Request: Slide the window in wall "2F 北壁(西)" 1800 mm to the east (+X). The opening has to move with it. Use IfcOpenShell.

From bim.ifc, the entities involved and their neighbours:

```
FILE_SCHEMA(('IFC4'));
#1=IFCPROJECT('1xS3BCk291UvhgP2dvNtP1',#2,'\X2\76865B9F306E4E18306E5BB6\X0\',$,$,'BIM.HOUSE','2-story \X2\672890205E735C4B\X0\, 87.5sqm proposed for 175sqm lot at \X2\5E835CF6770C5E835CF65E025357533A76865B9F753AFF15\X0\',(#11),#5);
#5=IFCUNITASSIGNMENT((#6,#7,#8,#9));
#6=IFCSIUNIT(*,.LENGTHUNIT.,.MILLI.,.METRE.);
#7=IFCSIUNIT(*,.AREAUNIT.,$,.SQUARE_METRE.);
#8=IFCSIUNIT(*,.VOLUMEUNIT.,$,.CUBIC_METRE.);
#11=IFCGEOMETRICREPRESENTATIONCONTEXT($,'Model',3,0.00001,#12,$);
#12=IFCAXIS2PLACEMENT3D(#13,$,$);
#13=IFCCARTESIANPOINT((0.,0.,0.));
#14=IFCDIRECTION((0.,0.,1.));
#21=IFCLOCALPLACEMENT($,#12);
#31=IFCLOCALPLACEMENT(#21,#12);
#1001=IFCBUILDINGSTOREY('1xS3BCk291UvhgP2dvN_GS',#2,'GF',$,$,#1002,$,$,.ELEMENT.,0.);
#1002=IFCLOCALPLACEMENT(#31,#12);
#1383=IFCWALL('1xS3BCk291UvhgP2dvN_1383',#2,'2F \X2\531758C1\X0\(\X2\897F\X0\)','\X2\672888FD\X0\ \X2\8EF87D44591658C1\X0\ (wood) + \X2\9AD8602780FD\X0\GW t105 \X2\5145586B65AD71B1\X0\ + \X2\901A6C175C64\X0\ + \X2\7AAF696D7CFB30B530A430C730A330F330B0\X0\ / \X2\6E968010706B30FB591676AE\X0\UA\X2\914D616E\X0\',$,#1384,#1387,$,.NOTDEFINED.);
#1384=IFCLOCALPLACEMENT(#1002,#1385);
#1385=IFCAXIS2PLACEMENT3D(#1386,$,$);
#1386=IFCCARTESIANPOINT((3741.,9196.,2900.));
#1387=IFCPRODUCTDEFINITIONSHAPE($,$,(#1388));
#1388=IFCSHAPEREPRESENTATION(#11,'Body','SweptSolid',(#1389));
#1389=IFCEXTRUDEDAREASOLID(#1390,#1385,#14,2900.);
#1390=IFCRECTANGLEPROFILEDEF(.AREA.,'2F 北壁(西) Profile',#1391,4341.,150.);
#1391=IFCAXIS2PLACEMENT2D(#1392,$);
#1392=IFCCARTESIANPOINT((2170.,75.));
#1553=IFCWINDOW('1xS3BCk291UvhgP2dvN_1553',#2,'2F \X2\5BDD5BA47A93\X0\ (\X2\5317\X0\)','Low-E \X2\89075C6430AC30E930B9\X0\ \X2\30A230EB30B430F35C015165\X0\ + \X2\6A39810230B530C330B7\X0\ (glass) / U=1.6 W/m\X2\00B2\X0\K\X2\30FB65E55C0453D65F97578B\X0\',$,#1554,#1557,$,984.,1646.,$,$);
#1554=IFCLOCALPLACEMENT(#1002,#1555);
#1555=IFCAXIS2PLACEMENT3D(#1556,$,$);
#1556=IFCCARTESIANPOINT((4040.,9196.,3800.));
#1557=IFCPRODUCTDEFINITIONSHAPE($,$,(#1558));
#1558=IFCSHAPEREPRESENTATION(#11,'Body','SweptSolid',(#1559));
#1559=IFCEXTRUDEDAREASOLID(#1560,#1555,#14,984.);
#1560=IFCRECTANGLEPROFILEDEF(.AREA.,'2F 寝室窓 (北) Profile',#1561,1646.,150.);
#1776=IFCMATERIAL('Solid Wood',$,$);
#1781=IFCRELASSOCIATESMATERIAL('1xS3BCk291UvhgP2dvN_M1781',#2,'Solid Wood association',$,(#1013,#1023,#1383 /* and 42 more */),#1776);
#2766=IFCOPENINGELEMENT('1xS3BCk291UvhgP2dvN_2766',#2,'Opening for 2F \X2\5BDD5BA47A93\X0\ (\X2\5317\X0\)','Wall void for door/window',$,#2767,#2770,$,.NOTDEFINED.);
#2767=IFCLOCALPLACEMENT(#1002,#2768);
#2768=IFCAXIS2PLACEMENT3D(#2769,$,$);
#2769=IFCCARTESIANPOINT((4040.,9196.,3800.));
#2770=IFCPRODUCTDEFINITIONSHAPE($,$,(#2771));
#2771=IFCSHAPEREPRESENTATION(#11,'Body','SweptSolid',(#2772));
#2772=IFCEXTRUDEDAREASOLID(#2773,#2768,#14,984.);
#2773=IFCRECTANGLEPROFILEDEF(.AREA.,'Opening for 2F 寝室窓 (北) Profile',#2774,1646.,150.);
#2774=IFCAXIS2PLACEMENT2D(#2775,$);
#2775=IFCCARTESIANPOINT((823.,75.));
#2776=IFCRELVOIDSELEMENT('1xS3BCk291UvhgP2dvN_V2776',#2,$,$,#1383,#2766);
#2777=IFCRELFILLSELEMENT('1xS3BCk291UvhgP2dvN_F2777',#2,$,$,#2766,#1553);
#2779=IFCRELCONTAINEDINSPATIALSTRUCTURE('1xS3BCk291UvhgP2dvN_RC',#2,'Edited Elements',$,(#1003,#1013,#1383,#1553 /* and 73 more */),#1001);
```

```python
import ifcopenshell
import ifcopenshell.api.geometry
import ifcopenshell.util.placement
import ifcopenshell.util.unit

model = ifcopenshell.open("bim.ifc")
unit_scale = ifcopenshell.util.unit.calculate_unit_scale(model)

window = model.by_guid("1xS3BCk291UvhgP2dvN_1553")
opening = window.FillsVoids[0].RelatingOpeningElement
wall = opening.VoidsElements[0].RelatingBuildingElement

wall_matrix = ifcopenshell.util.placement.get_local_placement(wall.ObjectPlacement)
shift = wall_matrix[:3, 0] * 1.8 / unit_scale
before = ifcopenshell.util.placement.get_local_placement(window.ObjectPlacement)[:3, 3].copy()

# The window is not placed relative to its opening, so move both.
for product in (opening, window):
    matrix = ifcopenshell.util.placement.get_local_placement(product.ObjectPlacement)
    matrix[:3, 3] += shift
    ifcopenshell.api.geometry.edit_object_placement(model, product=product, matrix=matrix, is_si=False)

after = ifcopenshell.util.placement.get_local_placement(window.ObjectPlacement)[:3, 3]
print("window moved by", (after - before).round(3) + 0.0)

model.write("bim_rev.ifc")
```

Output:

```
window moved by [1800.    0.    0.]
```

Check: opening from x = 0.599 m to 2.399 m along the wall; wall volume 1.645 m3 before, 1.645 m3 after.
